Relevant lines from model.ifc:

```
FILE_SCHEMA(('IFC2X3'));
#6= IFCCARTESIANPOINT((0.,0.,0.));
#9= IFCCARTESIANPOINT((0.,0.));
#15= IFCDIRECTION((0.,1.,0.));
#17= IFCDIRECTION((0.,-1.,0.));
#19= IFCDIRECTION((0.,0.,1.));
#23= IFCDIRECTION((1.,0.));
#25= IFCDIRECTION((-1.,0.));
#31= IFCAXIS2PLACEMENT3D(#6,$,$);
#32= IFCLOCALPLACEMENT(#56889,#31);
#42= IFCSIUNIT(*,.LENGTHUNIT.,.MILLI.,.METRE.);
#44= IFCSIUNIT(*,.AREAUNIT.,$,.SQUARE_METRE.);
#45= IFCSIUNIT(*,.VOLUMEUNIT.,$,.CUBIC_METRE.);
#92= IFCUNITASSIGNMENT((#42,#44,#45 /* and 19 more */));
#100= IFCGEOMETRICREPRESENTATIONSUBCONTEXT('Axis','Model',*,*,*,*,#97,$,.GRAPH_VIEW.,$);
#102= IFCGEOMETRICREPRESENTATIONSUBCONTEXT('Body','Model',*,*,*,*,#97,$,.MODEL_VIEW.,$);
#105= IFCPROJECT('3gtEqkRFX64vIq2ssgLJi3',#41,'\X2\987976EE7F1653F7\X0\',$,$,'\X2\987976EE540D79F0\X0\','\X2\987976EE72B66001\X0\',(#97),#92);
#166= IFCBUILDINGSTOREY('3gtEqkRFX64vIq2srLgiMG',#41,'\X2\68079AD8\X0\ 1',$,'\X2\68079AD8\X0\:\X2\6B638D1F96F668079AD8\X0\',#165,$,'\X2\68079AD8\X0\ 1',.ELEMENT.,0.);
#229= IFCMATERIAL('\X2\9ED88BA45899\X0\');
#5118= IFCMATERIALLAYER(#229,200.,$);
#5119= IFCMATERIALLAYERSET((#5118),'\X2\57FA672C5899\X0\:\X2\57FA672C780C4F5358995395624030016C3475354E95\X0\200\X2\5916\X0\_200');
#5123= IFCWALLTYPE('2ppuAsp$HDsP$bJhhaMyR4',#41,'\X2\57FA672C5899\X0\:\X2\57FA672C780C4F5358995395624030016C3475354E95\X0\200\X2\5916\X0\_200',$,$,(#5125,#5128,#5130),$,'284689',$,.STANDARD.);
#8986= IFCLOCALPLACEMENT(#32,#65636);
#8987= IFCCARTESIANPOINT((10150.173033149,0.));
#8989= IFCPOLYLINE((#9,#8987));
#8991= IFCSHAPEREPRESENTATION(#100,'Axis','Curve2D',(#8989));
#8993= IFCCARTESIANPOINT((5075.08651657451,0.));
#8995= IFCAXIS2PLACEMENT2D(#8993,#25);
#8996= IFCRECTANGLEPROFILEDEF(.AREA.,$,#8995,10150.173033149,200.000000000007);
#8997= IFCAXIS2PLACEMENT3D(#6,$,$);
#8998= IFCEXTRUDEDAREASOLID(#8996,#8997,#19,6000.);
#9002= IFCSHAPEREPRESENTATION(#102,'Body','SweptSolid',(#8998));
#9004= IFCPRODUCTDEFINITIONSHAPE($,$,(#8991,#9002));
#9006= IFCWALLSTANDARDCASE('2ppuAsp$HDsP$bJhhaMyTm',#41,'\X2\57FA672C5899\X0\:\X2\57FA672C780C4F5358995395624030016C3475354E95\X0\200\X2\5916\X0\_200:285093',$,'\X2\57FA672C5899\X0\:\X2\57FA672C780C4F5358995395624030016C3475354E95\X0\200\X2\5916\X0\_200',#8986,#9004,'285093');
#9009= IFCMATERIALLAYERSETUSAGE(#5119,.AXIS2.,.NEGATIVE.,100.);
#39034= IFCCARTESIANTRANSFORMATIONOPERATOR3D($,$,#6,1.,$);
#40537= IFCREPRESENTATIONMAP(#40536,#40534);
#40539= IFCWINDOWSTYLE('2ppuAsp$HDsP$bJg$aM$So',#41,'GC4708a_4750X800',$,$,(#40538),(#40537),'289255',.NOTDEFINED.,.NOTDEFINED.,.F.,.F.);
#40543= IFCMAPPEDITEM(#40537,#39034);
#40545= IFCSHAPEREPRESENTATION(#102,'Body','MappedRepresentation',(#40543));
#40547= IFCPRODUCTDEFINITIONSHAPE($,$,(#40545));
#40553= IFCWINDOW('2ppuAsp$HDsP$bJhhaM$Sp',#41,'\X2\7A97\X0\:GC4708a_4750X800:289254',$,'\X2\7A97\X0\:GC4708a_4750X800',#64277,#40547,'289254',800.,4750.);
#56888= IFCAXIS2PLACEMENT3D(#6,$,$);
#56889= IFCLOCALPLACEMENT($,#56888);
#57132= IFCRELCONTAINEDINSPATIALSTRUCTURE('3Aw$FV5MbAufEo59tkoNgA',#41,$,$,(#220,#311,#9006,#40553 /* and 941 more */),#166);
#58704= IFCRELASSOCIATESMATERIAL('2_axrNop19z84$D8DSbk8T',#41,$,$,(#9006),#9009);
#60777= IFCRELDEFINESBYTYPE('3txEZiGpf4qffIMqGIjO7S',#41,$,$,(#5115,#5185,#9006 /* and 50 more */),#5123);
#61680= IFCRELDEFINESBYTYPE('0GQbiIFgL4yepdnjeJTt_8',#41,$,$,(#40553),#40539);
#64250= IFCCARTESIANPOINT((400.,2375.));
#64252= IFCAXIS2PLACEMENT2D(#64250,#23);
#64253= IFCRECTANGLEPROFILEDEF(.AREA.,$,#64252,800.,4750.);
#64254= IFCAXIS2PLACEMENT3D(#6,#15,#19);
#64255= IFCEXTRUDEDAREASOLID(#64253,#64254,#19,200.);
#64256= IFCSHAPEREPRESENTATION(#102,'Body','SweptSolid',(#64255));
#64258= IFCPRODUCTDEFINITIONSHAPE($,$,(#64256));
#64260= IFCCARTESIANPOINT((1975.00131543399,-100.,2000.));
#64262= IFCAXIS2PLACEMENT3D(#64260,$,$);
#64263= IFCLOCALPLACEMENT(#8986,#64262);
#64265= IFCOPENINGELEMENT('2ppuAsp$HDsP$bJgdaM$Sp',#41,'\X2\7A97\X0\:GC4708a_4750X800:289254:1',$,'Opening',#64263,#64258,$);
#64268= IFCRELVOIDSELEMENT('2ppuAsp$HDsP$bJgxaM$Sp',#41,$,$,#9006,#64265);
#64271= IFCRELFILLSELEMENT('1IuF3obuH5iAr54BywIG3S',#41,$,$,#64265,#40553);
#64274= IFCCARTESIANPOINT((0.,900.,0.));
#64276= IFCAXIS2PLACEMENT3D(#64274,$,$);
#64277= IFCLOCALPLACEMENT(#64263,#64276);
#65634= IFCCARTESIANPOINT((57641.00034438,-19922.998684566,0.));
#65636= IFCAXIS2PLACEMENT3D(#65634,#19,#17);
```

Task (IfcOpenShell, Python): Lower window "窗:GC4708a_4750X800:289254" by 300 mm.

```python
import numpy as np
import ifcopenshell
import ifcopenshell.api.geometry
import ifcopenshell.util.placement
import ifcopenshell.util.unit

model = ifcopenshell.open("model.ifc")
unit_scale = ifcopenshell.util.unit.calculate_unit_scale(model)

window = model.by_guid("2ppuAsp$HDsP$bJhhaM$Sp")
opening = window.FillsVoids[0].RelatingOpeningElement
dz = -300.0

shift = np.array([0.0, 0.0, dz])
# The window is placed relative to its opening, so it follows when the opening moves.
matrix = ifcopenshell.util.placement.get_local_placement(opening.ObjectPlacement)
matrix[:3, 3] += shift
ifcopenshell.api.geometry.edit_object_placement(
    model, product=opening, matrix=matrix, is_si=False, should_transform_children=True
)

print(f"moved by {dz * unit_scale:+.3f} m")

model.write("model_v2.ifc")
```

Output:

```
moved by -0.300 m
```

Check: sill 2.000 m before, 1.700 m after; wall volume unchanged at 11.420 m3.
